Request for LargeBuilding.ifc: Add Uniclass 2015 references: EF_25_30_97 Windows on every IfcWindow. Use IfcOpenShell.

First a look at what the model holds.

```python
import ifcopenshell

model = ifcopenshell.open("LargeBuilding.ifc")
print(model.schema)
print("classifications:", [c.Name for c in model.by_type("IfcClassification")])
for ifc_class in ("IfcDoor", "IfcRoof", "IfcStair", "IfcWall", "IfcWindow"):
    print(ifc_class, len(model.by_type(ifc_class)))
```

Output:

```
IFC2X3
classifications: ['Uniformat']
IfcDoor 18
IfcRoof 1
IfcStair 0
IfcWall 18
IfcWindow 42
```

```python
import ifcopenshell
import ifcopenshell.api.classification

model = ifcopenshell.open("LargeBuilding.ifc")

# IFC2X3 requires Source and Edition and has no link from the project to the system.
system = model.create_entity("IfcClassification", Source="NBS", Edition="2015", Name="Uniclass 2015")

codes = {
    "IfcWindow": ("EF_25_30_97", "Windows"),
}
for ifc_class, (code, name) in codes.items():
    products = model.by_type(ifc_class)
    ifcopenshell.api.classification.add_reference(
        model, products=products, classification=system, identification=code, name=name
    )
    print(code, len(products))

model.write("LargeBuilding_rev.ifc")
```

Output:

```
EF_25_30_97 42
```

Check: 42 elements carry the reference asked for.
